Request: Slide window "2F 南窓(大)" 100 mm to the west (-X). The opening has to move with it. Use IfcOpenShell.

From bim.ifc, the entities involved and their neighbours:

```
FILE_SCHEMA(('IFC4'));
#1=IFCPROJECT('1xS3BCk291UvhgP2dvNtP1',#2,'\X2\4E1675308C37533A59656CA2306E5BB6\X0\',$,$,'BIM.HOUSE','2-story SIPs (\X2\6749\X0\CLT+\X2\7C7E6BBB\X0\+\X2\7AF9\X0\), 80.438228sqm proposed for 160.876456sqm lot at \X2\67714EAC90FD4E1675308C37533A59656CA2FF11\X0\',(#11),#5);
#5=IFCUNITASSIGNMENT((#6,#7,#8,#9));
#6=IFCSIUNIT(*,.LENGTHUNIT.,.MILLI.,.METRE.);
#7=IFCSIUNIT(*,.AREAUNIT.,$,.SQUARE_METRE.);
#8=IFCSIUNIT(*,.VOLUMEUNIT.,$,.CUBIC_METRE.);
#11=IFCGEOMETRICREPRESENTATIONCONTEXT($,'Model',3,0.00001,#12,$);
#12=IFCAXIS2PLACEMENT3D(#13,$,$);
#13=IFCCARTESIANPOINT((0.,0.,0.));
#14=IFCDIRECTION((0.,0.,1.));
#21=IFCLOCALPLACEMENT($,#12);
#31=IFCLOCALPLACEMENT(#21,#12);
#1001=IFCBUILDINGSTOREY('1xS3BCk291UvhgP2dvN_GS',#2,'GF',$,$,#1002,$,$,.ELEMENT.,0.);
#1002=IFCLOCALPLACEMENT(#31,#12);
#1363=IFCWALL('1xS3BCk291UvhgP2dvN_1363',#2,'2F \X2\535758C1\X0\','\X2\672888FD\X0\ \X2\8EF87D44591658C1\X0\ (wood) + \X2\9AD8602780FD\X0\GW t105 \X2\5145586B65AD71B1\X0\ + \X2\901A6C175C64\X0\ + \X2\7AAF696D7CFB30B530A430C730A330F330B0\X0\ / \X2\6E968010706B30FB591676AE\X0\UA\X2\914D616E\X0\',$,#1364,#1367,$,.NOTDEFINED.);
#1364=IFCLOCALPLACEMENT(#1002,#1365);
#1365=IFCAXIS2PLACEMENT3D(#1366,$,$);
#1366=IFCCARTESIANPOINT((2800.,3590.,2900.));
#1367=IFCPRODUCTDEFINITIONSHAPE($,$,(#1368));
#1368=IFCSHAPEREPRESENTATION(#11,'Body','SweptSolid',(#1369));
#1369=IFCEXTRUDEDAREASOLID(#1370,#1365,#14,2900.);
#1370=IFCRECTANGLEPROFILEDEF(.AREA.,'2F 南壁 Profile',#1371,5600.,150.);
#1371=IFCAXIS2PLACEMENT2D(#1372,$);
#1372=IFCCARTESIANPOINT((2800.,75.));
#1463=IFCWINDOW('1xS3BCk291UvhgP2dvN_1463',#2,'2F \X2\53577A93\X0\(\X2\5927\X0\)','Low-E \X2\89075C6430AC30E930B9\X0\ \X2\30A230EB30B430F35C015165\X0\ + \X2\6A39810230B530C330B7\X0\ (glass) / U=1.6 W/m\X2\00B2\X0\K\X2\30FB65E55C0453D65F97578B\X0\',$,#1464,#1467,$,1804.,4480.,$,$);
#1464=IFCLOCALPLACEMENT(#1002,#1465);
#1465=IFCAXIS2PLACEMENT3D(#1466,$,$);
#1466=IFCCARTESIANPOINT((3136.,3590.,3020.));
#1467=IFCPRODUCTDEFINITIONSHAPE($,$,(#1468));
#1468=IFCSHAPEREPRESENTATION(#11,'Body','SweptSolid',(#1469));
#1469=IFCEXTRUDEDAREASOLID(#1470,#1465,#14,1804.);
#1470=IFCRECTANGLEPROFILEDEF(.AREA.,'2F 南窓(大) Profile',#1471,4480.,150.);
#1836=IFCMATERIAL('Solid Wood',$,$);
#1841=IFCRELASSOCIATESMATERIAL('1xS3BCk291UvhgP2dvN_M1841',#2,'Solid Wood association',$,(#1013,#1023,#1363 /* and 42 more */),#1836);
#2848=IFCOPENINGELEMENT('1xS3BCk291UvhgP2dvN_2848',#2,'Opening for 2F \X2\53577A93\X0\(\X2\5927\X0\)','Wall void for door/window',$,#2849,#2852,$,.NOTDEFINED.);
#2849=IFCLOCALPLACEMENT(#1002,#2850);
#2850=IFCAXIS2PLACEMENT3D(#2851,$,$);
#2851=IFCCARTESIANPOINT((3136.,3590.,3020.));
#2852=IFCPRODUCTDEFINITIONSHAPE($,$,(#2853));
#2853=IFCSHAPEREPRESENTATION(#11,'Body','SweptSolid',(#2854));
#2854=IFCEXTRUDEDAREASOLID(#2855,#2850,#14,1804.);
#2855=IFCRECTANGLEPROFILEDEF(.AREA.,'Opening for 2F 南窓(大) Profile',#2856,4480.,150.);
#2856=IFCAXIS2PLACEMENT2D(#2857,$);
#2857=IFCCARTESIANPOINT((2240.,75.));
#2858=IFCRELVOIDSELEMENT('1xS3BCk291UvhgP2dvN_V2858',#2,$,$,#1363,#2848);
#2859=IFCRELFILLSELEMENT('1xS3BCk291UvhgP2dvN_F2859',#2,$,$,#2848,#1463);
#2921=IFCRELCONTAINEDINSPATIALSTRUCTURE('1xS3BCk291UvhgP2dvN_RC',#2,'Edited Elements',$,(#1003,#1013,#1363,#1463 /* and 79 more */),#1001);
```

```python
import ifcopenshell
import ifcopenshell.api.geometry
import ifcopenshell.util.placement

model = ifcopenshell.open("bim.ifc")

window = model.by_id(1463)
opening = window.FillsVoids[0].RelatingOpeningElement
wall = opening.VoidsElements[0].RelatingBuildingElement

wall_matrix = ifcopenshell.util.placement.get_local_placement(wall.ObjectPlacement)
shift = wall_matrix[:3, 0] * -100.0
before = ifcopenshell.util.placement.get_local_placement(window.ObjectPlacement)[:3, 3].copy()

# The window is not placed relative to its opening, so move both.
for product in (opening, window):
    matrix = ifcopenshell.util.placement.get_local_placement(product.ObjectPlacement)
    matrix[:3, 3] += shift
    ifcopenshell.api.geometry.edit_object_placement(model, product=product, matrix=matrix, is_si=False)

after = ifcopenshell.util.placement.get_local_placement(window.ObjectPlacement)[:3, 3]
print("window moved by", (after - before).round(3) + 0.0)

model.write("bim_v2.ifc")
```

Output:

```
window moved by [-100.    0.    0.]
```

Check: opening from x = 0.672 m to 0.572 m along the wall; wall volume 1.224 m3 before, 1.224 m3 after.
